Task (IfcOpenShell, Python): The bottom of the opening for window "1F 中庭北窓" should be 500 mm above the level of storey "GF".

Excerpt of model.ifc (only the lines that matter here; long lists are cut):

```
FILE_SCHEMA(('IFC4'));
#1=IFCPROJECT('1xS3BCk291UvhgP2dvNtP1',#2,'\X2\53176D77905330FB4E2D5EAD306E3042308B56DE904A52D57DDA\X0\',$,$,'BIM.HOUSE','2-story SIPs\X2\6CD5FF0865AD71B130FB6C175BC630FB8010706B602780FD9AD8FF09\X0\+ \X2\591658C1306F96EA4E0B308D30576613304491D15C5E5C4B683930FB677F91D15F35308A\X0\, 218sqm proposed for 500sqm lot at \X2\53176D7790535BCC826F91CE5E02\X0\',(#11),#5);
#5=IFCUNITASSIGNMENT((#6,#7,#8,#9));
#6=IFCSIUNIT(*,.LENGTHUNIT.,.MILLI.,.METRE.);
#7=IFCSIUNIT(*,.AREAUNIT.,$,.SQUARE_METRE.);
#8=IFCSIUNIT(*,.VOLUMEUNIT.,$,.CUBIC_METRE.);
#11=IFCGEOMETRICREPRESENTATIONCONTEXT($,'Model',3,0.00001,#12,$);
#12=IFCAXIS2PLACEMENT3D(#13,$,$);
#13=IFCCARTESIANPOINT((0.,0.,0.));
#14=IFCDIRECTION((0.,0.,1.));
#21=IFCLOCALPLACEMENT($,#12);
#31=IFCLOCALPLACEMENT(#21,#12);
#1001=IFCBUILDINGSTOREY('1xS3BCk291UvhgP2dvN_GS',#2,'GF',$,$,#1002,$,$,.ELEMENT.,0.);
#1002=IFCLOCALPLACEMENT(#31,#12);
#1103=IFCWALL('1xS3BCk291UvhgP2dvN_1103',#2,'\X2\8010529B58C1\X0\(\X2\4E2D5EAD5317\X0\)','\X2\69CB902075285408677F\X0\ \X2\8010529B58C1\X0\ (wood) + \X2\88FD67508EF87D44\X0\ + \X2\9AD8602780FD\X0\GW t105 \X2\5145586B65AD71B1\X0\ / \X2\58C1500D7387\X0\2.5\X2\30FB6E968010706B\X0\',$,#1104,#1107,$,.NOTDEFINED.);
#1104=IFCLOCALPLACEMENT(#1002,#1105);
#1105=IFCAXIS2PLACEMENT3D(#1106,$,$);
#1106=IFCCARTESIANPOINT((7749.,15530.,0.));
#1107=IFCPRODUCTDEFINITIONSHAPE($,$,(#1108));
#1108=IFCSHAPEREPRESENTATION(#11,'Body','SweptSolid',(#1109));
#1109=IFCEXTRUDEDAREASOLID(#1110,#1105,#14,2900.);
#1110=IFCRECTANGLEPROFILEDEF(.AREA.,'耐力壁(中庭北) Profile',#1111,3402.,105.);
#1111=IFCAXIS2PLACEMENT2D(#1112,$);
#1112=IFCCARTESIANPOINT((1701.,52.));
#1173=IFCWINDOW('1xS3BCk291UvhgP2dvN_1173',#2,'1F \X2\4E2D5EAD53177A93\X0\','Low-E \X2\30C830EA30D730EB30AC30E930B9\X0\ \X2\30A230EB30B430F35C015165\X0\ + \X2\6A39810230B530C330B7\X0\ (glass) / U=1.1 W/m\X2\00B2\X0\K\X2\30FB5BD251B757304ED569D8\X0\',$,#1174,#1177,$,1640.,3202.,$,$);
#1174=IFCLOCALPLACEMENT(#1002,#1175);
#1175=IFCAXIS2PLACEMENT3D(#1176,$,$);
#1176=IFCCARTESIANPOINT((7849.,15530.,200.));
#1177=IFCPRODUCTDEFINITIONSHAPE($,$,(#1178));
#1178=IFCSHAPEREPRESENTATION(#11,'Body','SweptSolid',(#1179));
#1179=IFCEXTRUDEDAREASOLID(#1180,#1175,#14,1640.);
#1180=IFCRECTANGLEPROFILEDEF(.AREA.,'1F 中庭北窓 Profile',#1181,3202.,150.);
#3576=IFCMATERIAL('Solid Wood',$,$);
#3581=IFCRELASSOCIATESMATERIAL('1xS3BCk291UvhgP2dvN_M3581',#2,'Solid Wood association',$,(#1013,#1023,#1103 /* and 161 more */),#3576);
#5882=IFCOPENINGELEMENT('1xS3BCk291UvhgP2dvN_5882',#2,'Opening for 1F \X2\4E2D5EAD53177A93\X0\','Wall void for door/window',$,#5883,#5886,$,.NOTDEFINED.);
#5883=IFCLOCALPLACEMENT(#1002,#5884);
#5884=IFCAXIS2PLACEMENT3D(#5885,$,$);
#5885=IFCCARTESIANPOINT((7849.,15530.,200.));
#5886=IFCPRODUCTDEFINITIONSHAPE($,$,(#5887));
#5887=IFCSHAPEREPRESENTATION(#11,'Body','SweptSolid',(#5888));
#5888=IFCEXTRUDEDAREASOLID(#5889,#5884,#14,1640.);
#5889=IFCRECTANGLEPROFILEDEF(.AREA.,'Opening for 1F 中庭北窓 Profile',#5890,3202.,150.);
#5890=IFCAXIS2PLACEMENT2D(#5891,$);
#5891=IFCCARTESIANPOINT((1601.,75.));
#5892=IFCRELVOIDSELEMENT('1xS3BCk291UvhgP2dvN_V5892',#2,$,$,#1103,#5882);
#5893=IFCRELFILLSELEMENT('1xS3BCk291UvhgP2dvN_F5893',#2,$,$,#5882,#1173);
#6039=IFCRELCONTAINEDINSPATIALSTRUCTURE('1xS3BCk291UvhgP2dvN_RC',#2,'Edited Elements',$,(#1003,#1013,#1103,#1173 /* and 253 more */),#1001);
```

```python
import numpy as np
import ifcopenshell
import ifcopenshell.api.geometry
import ifcopenshell.geom
import ifcopenshell.util.element
import ifcopenshell.util.placement
import ifcopenshell.util.shape
import ifcopenshell.util.unit

model = ifcopenshell.open("model.ifc")
unit_scale = ifcopenshell.util.unit.calculate_unit_scale(model)

window = model.by_guid("1xS3BCk291UvhgP2dvN_1173")
opening = window.FillsVoids[0].RelatingOpeningElement
storey = ifcopenshell.util.element.get_container(window, ifc_class="IfcBuildingStorey")
level = ifcopenshell.util.placement.get_local_placement(storey.ObjectPlacement)[2, 3]

# The opening's origin need not be at the sill, so measure its lowest point.
shape = ifcopenshell.geom.create_shape(ifcopenshell.geom.settings(), opening)
bottom = ifcopenshell.util.shape.get_shape_bottom_elevation(shape, shape.geometry) / unit_scale
dz = level + 0.5 / unit_scale - bottom

shift = np.array([0.0, 0.0, dz])
# The window is not placed relative to its opening, so move both.
for product in (opening, window):
    matrix = ifcopenshell.util.placement.get_local_placement(product.ObjectPlacement)
    matrix[:3, 3] += shift
    ifcopenshell.api.geometry.edit_object_placement(model, product=product, matrix=matrix, is_si=False)

print(f"moved by {dz * unit_scale:+.3f} m")

model.write("model_updated.ifc")
```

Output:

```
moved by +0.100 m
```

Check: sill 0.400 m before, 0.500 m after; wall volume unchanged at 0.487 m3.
